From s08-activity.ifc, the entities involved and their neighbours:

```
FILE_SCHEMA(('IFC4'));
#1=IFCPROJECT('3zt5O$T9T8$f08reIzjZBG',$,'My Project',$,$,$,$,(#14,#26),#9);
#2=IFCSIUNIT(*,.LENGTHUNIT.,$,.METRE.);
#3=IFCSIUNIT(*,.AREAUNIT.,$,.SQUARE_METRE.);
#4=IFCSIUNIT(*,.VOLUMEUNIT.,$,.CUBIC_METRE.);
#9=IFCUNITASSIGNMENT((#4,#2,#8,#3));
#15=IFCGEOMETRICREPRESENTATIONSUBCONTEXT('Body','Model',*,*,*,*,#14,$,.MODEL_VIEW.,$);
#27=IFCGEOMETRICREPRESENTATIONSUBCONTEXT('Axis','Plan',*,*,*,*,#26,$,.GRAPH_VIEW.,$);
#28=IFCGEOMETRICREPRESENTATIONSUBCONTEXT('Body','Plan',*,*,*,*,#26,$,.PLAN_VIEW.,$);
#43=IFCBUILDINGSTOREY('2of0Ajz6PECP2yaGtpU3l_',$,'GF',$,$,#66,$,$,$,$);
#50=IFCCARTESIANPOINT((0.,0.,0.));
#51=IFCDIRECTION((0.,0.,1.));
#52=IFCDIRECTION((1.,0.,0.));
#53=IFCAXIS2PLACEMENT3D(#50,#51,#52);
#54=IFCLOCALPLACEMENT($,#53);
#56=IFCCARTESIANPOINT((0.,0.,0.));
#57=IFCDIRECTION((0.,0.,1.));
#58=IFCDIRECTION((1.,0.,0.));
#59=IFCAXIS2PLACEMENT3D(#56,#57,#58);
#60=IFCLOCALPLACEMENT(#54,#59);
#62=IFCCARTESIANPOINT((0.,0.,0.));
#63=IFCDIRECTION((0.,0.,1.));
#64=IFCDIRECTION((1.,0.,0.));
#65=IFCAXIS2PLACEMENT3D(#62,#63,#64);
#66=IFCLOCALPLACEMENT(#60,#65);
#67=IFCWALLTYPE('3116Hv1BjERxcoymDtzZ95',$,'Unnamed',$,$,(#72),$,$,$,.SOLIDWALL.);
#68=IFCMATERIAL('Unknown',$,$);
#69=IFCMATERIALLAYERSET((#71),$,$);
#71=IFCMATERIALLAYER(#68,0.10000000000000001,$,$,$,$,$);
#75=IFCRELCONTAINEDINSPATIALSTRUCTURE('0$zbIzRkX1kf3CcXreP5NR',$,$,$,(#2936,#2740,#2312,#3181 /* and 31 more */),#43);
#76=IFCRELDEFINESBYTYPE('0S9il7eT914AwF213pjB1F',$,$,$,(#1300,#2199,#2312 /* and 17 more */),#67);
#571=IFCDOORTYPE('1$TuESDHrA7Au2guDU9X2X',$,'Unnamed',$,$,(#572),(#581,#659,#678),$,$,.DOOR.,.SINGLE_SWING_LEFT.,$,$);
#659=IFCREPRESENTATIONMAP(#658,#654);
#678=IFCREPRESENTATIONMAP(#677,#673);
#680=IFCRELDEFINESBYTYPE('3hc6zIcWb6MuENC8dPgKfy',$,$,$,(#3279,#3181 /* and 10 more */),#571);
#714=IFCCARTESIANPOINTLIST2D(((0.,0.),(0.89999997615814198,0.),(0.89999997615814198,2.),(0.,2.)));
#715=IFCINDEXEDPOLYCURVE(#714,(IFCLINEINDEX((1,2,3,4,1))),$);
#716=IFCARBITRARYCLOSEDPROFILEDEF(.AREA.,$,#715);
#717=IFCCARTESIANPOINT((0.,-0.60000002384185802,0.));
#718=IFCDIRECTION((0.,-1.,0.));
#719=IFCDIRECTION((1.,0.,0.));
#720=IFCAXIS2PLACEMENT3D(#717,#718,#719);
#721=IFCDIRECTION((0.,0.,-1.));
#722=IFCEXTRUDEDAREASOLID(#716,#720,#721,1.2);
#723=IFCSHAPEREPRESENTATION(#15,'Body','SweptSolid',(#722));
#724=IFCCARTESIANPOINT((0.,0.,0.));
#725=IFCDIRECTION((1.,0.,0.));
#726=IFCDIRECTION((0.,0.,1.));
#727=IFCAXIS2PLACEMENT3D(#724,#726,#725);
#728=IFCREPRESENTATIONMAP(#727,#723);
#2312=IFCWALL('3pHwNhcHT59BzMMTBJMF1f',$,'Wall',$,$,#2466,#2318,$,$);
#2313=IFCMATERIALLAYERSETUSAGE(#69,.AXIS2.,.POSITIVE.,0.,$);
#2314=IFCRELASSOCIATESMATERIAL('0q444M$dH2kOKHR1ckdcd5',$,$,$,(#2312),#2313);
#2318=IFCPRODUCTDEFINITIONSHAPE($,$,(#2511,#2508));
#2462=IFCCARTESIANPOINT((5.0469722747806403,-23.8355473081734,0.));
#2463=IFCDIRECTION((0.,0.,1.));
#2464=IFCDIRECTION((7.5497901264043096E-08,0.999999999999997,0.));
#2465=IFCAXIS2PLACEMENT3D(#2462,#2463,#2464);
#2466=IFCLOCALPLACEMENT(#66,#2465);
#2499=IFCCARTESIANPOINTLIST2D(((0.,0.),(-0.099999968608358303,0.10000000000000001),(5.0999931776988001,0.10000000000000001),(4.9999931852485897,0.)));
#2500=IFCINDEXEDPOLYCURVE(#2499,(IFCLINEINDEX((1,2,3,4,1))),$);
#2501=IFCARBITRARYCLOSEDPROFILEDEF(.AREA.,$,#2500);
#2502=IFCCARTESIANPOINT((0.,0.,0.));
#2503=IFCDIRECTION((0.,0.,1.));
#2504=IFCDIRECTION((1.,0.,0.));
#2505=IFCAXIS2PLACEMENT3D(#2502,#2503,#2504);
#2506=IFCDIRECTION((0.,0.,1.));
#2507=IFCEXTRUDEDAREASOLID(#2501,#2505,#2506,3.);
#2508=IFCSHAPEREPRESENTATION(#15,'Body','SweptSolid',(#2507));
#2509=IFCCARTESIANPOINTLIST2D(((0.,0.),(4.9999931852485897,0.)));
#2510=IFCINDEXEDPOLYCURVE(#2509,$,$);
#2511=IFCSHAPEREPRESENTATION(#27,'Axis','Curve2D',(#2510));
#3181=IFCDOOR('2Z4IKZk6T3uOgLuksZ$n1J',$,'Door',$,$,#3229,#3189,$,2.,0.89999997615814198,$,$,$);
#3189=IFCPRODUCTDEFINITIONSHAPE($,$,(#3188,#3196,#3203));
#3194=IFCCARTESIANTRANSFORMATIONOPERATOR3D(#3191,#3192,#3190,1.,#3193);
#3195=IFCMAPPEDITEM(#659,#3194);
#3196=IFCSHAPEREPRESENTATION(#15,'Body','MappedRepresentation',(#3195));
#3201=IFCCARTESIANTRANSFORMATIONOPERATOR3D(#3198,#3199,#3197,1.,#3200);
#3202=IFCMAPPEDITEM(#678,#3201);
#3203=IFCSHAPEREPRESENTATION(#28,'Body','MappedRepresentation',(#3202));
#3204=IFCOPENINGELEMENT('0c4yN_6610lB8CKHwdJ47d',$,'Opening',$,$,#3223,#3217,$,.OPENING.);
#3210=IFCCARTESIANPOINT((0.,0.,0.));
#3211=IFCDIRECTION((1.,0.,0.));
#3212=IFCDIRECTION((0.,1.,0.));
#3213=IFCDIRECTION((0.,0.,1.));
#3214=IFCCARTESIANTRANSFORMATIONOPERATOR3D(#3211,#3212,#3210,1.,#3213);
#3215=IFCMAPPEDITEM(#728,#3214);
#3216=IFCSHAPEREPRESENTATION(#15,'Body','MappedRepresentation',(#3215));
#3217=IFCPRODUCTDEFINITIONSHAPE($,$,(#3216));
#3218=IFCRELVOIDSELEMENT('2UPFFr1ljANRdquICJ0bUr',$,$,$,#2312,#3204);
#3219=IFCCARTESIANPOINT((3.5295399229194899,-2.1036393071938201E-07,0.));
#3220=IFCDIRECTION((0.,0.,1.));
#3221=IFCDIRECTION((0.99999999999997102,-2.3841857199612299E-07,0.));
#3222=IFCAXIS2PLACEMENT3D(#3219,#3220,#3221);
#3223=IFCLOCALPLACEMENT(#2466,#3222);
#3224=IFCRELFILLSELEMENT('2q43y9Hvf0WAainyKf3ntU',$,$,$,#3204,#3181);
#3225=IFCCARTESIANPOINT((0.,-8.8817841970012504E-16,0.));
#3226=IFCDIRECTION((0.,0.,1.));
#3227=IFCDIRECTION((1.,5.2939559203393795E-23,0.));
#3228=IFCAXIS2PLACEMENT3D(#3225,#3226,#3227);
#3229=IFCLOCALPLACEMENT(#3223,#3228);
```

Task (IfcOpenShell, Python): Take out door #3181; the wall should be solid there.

```python
import ifcopenshell
import ifcopenshell.api.feature
import ifcopenshell.api.root
import ifcopenshell.geom
import ifcopenshell.util.shape

model = ifcopenshell.open("s08-activity.ifc")
settings = ifcopenshell.geom.settings()


def volume(element):
    """Net volume in cubic metres, openings subtracted."""
    shape = ifcopenshell.geom.create_shape(settings, element)
    return ifcopenshell.util.shape.get_volume(shape.geometry)


door = model.by_id(3181)
opening = door.FillsVoids[0].RelatingOpeningElement
wall = opening.VoidsElements[0].RelatingBuildingElement
before = volume(wall)

ifcopenshell.api.root.remove_product(model, product=door)
ifcopenshell.api.feature.remove_feature(model, feature=opening)

after = volume(wall)

print(f"wall volume {before:.3f} -> {after:.3f} m3")

model.write("s08-activity_updated.ifc")
```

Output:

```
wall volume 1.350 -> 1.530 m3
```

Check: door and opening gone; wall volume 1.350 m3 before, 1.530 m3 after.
